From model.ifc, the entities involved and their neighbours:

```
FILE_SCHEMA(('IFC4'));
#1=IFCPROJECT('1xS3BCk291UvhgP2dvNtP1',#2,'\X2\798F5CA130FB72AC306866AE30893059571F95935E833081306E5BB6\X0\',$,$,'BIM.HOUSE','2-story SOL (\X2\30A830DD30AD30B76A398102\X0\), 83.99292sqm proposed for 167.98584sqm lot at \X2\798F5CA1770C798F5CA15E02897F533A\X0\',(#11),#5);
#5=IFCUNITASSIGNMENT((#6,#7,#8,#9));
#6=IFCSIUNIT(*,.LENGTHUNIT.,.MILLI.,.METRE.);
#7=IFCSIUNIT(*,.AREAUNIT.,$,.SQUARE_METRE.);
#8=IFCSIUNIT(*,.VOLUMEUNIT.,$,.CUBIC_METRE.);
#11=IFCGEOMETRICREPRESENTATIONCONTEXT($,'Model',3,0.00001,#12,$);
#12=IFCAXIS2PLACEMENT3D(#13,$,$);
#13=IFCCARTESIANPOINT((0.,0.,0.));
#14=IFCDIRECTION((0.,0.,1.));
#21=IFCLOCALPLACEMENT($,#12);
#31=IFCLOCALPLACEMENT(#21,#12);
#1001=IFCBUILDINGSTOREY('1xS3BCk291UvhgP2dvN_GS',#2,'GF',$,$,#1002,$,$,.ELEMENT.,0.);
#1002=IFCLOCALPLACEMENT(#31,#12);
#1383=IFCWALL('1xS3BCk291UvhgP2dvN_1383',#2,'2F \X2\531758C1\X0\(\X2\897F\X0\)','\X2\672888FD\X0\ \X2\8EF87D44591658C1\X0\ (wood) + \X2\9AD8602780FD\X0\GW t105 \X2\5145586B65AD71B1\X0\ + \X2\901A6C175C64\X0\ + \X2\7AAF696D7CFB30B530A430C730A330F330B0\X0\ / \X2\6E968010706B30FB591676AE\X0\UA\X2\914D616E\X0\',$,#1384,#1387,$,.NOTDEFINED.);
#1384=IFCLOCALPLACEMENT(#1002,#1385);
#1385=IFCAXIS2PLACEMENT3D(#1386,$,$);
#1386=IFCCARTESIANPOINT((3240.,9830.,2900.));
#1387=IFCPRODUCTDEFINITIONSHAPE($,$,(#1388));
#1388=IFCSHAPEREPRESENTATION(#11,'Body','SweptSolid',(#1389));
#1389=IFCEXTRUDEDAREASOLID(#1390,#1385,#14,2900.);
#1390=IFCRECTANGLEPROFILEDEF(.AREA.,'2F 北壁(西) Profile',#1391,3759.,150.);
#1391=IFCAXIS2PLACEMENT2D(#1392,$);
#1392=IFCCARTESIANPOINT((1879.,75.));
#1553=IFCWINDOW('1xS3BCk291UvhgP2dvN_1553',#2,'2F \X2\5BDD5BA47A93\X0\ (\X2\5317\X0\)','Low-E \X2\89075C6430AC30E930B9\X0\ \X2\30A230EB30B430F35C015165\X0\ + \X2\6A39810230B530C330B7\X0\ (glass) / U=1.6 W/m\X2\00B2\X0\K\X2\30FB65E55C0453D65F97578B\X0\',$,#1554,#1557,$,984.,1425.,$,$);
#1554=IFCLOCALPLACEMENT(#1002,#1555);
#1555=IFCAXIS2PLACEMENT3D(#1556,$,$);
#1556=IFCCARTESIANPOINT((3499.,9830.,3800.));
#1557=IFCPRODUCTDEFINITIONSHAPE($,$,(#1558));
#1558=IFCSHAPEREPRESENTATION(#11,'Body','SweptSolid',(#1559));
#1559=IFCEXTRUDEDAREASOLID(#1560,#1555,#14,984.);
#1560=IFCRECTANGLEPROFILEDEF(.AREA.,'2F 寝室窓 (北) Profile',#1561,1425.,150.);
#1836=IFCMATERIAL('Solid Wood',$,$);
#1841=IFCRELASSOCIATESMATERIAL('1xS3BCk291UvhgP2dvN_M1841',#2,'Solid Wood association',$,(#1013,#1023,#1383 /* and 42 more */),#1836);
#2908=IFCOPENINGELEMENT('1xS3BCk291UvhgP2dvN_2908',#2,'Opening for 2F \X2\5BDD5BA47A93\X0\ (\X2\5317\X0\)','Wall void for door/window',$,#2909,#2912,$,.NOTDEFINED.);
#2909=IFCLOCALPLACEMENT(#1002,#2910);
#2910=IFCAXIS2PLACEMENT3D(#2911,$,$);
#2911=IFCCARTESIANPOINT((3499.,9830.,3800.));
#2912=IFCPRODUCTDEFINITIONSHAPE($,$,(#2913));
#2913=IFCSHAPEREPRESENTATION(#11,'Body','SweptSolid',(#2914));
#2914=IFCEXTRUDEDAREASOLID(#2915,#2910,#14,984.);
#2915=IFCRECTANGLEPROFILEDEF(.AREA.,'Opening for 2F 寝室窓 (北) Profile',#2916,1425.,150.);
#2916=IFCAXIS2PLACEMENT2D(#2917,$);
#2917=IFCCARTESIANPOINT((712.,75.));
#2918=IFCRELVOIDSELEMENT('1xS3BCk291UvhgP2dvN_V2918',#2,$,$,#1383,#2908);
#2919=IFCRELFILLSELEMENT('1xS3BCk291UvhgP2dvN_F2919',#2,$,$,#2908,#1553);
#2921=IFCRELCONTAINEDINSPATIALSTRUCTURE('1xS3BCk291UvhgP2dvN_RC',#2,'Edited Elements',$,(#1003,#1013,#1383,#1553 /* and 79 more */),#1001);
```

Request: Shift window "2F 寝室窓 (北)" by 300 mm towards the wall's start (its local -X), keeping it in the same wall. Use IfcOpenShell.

```python
import ifcopenshell
import ifcopenshell.api.geometry
import ifcopenshell.util.placement
import ifcopenshell.util.unit

model = ifcopenshell.open("model.ifc")
unit_scale = ifcopenshell.util.unit.calculate_unit_scale(model)

window = model.by_guid("1xS3BCk291UvhgP2dvN_1553")
opening = window.FillsVoids[0].RelatingOpeningElement
wall = opening.VoidsElements[0].RelatingBuildingElement

wall_matrix = ifcopenshell.util.placement.get_local_placement(wall.ObjectPlacement)
shift = wall_matrix[:3, 0] * -0.3 / unit_scale
before = ifcopenshell.util.placement.get_local_placement(window.ObjectPlacement)[:3, 3].copy()

# The window is not placed relative to its opening, so move both.
for product in (opening, window):
    matrix = ifcopenshell.util.placement.get_local_placement(product.ObjectPlacement)
    matrix[:3, 3] += shift
    ifcopenshell.api.geometry.edit_object_placement(model, product=product, matrix=matrix, is_si=False)

after = ifcopenshell.util.placement.get_local_placement(window.ObjectPlacement)[:3, 3]
print("window moved by", (after - before).round(3) + 0.0)

model.write("model_v2.ifc")
```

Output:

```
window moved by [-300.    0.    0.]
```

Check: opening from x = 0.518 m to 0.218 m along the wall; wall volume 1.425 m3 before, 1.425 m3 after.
